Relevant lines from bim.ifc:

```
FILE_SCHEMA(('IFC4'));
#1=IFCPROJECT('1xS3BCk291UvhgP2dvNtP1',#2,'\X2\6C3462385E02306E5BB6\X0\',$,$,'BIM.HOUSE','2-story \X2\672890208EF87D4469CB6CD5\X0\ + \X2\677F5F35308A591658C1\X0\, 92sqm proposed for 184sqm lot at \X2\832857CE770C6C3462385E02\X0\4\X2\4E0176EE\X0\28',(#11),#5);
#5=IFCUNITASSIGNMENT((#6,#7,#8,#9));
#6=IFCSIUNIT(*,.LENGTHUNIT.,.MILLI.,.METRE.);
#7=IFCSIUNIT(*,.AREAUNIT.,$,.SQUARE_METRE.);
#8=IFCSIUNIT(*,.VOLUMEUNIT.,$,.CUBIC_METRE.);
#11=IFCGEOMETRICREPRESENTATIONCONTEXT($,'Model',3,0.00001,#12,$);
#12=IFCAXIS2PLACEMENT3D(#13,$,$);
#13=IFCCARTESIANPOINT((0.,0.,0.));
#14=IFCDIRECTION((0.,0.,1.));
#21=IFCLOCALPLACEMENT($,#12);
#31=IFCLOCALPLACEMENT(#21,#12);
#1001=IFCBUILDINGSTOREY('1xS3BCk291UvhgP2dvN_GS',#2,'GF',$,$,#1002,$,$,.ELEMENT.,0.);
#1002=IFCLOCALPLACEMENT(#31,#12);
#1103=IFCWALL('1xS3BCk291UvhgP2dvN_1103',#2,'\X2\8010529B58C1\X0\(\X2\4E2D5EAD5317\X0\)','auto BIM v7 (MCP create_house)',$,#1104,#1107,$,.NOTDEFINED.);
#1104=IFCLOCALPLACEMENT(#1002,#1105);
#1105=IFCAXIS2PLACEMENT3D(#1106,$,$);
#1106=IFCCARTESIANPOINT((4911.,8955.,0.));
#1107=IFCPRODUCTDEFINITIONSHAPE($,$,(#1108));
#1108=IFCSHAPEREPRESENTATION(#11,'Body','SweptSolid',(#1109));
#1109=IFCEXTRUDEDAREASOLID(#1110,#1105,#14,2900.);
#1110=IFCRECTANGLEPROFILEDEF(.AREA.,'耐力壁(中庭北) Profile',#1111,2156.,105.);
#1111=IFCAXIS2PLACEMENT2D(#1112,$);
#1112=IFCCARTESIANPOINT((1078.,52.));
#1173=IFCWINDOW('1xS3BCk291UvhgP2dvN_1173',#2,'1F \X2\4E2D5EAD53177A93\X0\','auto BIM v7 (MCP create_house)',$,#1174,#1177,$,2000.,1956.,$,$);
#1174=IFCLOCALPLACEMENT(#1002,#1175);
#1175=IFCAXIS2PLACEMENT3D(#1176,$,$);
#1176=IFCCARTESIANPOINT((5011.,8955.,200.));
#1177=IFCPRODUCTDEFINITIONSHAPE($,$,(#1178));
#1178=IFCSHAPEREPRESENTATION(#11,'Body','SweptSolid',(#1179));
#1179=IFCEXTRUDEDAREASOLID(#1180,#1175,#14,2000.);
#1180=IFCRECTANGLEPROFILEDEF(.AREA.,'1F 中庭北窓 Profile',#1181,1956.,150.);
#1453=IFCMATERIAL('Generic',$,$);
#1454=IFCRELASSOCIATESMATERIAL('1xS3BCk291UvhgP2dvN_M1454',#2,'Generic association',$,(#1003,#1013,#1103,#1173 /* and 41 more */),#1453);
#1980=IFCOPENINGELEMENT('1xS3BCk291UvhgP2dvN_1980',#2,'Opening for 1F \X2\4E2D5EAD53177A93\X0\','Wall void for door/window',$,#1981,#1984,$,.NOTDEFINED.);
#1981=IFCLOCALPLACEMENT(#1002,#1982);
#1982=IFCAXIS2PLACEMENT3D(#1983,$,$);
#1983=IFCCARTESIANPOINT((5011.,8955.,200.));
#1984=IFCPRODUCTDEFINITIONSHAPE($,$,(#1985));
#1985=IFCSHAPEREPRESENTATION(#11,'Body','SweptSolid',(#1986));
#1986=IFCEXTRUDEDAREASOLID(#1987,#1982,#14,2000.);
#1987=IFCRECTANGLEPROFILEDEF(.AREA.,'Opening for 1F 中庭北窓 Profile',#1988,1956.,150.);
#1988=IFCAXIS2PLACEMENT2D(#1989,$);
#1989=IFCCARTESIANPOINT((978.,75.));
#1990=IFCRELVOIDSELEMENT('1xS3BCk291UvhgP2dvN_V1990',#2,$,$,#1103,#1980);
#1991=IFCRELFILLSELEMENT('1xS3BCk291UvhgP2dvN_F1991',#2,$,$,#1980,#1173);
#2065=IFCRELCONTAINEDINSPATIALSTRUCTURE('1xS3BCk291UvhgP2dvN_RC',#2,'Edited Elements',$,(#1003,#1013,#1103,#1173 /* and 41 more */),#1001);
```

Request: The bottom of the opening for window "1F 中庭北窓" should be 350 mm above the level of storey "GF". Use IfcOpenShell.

```python
import numpy as np
import ifcopenshell
import ifcopenshell.api.geometry
import ifcopenshell.geom
import ifcopenshell.util.element
import ifcopenshell.util.placement
import ifcopenshell.util.shape
import ifcopenshell.util.unit

model = ifcopenshell.open("bim.ifc")
unit_scale = ifcopenshell.util.unit.calculate_unit_scale(model)

window = model.by_guid("1xS3BCk291UvhgP2dvN_1173")
opening = window.FillsVoids[0].RelatingOpeningElement
storey = ifcopenshell.util.element.get_container(window, ifc_class="IfcBuildingStorey")
level = ifcopenshell.util.placement.get_local_placement(storey.ObjectPlacement)[2, 3]

# The opening's origin need not be at the sill, so measure its lowest point.
shape = ifcopenshell.geom.create_shape(ifcopenshell.geom.settings(), opening)
bottom = ifcopenshell.util.shape.get_shape_bottom_elevation(shape, shape.geometry) / unit_scale
dz = level + 0.35 / unit_scale - bottom

shift = np.array([0.0, 0.0, dz])
# The window is not placed relative to its opening, so move both.
for product in (opening, window):
    matrix = ifcopenshell.util.placement.get_local_placement(product.ObjectPlacement)
    matrix[:3, 3] += shift
    ifcopenshell.api.geometry.edit_object_placement(model, product=product, matrix=matrix, is_si=False)

print(f"moved by {dz * unit_scale:+.3f} m")

model.write("bim_updated.ifc")
```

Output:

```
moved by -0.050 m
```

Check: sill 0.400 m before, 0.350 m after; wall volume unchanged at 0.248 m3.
